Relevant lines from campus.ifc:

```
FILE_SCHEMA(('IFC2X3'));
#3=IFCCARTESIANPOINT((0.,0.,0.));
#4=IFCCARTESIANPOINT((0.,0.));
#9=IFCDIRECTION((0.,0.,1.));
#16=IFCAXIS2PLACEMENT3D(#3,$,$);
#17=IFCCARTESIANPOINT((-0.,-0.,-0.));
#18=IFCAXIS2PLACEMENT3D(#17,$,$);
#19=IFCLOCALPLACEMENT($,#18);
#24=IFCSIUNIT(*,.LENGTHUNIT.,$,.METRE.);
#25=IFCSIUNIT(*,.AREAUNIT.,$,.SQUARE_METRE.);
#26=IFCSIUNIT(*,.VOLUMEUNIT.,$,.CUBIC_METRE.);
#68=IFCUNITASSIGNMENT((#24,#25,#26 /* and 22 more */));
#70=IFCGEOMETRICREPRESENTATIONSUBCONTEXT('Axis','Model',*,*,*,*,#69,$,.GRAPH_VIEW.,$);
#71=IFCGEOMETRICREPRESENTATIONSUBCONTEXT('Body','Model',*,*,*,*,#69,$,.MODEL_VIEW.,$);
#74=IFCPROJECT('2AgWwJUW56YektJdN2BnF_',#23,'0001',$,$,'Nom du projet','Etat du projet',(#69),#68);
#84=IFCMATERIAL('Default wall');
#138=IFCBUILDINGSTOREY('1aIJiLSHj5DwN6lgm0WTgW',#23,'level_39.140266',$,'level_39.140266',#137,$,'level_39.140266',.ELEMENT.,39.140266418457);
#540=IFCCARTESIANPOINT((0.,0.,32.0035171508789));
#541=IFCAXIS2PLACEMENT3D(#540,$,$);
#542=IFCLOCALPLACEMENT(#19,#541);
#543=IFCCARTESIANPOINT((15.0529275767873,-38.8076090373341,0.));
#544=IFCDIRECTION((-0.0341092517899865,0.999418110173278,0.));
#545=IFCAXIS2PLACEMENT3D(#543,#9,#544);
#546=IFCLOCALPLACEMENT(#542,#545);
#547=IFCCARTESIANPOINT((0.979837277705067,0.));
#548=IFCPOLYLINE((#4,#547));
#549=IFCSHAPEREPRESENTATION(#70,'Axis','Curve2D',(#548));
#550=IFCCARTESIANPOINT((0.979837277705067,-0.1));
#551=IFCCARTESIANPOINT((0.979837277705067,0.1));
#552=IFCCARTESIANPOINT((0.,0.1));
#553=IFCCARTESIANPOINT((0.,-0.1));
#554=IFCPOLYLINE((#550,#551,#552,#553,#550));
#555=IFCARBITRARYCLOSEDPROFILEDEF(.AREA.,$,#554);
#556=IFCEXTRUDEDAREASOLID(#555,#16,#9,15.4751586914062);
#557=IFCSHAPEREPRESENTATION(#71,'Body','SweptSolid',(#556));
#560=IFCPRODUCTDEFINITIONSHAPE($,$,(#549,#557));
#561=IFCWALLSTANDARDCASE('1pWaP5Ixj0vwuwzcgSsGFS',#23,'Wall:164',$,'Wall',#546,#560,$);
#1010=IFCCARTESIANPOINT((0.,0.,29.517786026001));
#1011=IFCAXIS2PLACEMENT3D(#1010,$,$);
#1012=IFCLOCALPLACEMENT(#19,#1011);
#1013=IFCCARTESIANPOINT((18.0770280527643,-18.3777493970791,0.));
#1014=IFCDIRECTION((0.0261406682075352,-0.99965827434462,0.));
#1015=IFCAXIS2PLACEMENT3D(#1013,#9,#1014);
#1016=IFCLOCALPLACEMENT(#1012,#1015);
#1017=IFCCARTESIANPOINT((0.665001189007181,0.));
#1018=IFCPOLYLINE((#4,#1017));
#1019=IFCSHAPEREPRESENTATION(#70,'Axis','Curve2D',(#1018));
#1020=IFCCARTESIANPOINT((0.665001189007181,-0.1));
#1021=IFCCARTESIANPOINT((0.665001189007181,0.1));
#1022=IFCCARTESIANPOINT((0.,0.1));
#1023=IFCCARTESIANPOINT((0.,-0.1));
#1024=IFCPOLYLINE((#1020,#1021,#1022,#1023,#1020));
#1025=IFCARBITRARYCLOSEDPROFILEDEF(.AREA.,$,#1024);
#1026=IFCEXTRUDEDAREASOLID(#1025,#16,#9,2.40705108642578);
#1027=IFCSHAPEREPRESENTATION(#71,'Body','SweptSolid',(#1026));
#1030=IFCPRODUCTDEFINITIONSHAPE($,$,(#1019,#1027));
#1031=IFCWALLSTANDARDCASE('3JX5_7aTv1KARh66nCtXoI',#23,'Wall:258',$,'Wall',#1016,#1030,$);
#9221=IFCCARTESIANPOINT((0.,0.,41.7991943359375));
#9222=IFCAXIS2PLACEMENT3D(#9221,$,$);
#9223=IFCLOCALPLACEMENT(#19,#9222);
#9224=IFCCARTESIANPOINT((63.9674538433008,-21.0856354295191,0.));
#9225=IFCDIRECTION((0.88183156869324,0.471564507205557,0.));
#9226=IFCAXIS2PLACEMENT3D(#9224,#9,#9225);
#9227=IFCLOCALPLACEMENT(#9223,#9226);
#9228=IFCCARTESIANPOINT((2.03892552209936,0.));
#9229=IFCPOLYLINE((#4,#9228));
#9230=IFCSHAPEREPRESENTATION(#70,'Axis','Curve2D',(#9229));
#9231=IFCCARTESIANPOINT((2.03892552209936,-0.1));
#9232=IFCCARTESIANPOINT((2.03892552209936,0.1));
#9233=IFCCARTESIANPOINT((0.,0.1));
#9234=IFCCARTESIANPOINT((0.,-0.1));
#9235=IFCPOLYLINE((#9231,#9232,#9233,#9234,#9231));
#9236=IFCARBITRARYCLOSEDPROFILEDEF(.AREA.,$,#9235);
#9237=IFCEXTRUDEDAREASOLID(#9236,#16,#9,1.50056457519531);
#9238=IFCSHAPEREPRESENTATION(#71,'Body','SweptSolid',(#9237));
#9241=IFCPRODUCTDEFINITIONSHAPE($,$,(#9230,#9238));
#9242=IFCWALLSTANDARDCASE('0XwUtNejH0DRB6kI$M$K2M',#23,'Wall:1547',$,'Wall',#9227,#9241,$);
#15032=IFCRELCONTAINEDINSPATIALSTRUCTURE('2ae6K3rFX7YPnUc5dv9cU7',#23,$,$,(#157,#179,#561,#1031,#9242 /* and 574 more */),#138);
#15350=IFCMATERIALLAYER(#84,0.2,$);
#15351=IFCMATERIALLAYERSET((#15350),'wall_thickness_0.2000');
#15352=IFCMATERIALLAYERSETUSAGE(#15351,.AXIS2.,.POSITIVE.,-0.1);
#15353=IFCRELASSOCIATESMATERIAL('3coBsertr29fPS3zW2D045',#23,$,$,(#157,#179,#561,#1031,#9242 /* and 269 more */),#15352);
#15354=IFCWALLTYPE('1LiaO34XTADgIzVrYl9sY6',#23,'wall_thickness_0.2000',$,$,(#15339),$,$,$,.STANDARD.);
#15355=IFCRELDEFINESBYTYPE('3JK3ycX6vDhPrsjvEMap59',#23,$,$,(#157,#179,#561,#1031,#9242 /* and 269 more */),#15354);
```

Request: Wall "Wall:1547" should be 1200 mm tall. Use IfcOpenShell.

```python
import ifcopenshell
import ifcopenshell.geom
import ifcopenshell.util.representation
import ifcopenshell.util.shape

model = ifcopenshell.open("campus.ifc")
settings = ifcopenshell.geom.settings()


def volume(element):
    """Net volume in cubic metres, openings subtracted."""
    shape = ifcopenshell.geom.create_shape(settings, element)
    return ifcopenshell.util.shape.get_volume(shape.geometry)


wall = model.by_guid("0XwUtNejH0DRB6kI$M$K2M")
before = volume(wall)

body = ifcopenshell.util.representation.get_representation(wall, "Model", "Body")
solid = body.Items[0]
old_height = solid.Depth
solid.Depth = 1.2
after = volume(wall)

print(f"height {old_height:g} -> {solid.Depth:g}, volume {before:.3f} -> {after:.3f} m3")

model.write("campus-out.ifc")
```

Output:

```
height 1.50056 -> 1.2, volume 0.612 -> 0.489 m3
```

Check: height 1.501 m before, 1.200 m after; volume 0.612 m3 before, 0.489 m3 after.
